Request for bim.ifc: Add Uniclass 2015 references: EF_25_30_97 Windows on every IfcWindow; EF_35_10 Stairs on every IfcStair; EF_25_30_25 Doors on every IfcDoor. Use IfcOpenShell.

First a look at what the model holds.

```python
import ifcopenshell

model = ifcopenshell.open("bim.ifc")
print(model.schema)
print("classifications:", [c.Name for c in model.by_type("IfcClassification")])
for ifc_class in ("IfcDoor", "IfcRoof", "IfcStair", "IfcWall", "IfcWindow"):
    print(ifc_class, len(model.by_type(ifc_class)))
```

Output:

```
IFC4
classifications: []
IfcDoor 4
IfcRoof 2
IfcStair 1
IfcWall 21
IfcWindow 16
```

```python
import ifcopenshell
import ifcopenshell.api.classification

model = ifcopenshell.open("bim.ifc")

system = ifcopenshell.api.classification.add_classification(model, classification="Uniclass 2015")

codes = {
    "IfcWindow": ("EF_25_30_97", "Windows"),
    "IfcStair": ("EF_35_10", "Stairs"),
    "IfcDoor": ("EF_25_30_25", "Doors"),
}
for ifc_class, (code, name) in codes.items():
    products = model.by_type(ifc_class)
    ifcopenshell.api.classification.add_reference(
        model, products=products, classification=system, identification=code, name=name
    )
    print(code, len(products))

model.write("bim_rev.ifc")
```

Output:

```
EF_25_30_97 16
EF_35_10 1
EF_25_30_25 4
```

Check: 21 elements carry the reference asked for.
